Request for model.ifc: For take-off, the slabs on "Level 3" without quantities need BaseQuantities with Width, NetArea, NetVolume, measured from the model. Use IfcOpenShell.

First a look at what the model holds.

```python
import ifcopenshell
import ifcopenshell.util.element
import ifcopenshell.util.unit

model = ifcopenshell.open("model.ifc")
print(model.schema)
for unit_type in ("LENGTHUNIT", "AREAUNIT", "VOLUMEUNIT"):
    print(unit_type, ifcopenshell.util.unit.calculate_unit_scale(model, unit_type))
storey = next(s for s in model.by_type("IfcBuildingStorey") if s.Name == "Level 3")
slabs = [e for e in ifcopenshell.util.element.get_decomposition(storey) if e.is_a("IfcSlab")]
for e in sorted(slabs, key=lambda e: e.id()):
    print(e.id(), e.is_a(), e.Name, list(ifcopenshell.util.element.get_psets(e, qtos_only=True)), sep=" | ")
```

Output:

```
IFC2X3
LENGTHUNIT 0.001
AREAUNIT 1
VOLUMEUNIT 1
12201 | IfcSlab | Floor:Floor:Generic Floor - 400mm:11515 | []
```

```python
import ifcopenshell
import ifcopenshell.api.pset
import ifcopenshell.geom
import ifcopenshell.util.element
import ifcopenshell.util.shape
import ifcopenshell.util.unit

model = ifcopenshell.open("model.ifc")
unit_scale = ifcopenshell.util.unit.calculate_unit_scale(model)
area_scale = ifcopenshell.util.unit.calculate_unit_scale(model, "AREAUNIT")
volume_scale = ifcopenshell.util.unit.calculate_unit_scale(model, "VOLUMEUNIT")
settings = ifcopenshell.geom.settings()

storey = next(s for s in model.by_type("IfcBuildingStorey") if s.Name == "Level 3")
slabs = [e for e in ifcopenshell.util.element.get_decomposition(storey) if e.is_a("IfcSlab")]

for e in sorted(slabs, key=lambda e: e.id()):
    if ifcopenshell.util.element.get_psets(e, qtos_only=True, should_inherit=False):
        continue
    # Geometry comes back in metres, in the element's own axes.
    shape = ifcopenshell.geom.create_shape(settings, e)
    values = {
        "Width": ifcopenshell.util.shape.get_z(shape.geometry) / unit_scale,
        "NetArea": ifcopenshell.util.shape.get_footprint_area(shape.geometry) / area_scale,
        "NetVolume": ifcopenshell.util.shape.get_volume(shape.geometry) / volume_scale,
    }
    qto = ifcopenshell.api.pset.add_qto(model, product=e, name="BaseQuantities")
    ifcopenshell.api.pset.edit_qto(model, qto=qto, properties=values)
    print(e.id(), {k: round(v, 3) for k, v in values.items()})

model.write("model_edited.ifc")
```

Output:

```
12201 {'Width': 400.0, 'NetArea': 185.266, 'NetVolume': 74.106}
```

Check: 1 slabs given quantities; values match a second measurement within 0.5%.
